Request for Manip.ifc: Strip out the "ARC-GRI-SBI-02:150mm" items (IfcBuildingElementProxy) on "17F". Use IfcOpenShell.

First a look at what the model holds.

```python
import ifcopenshell
import ifcopenshell.util.element

model = ifcopenshell.open("Manip.ifc")
print(model.schema)
storey = next(s for s in model.by_type("IfcBuildingStorey") if s.Name == "17F")
proxies = [e for e in ifcopenshell.util.element.get_decomposition(storey) if e.is_a("IfcBuildingElementProxy")]
seen = {}
for e in proxies:
    element_type = ifcopenshell.util.element.get_type(e)
    name = element_type.Name if element_type not in (None, e) else None
    seen[name] = seen.get(name, 0) + 1
for name, count in sorted(seen.items(), key=str):
    print(count, "x", name)
```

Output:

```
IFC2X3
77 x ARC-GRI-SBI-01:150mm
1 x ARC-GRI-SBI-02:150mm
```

```python
import ifcopenshell
import ifcopenshell.api.root
import ifcopenshell.util.element

model = ifcopenshell.open("Manip.ifc")

storey = next(s for s in model.by_type("IfcBuildingStorey") if s.Name == "17F")
proxies = [e for e in ifcopenshell.util.element.get_decomposition(storey) if e.is_a("IfcBuildingElementProxy")]
targets = [e for e in proxies if (t := ifcopenshell.util.element.get_type(e)) not in (None, e) and t.Name == "ARC-GRI-SBI-02:150mm"]

for e in targets:
    ifcopenshell.api.root.remove_product(model, product=e)
print(len(targets), "removed")

model.write("Manip_updated.ifc")
```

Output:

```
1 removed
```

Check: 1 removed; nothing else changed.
